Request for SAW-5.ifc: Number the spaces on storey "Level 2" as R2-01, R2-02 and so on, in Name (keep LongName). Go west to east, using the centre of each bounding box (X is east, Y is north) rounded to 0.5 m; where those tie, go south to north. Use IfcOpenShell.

First a look at what the model holds.

```python
import ifcopenshell
import ifcopenshell.util.element
import ifcopenshell.util.placement

model = ifcopenshell.open("SAW-5.ifc")
print(model.schema)
storey = next(s for s in model.by_type("IfcBuildingStorey") if s.Name == "Level 2")
spaces = [e for e in ifcopenshell.util.element.get_decomposition(storey) if e.is_a("IfcSpace")]
for e in sorted(spaces, key=lambda e: e.id()):
    origin = ifcopenshell.util.placement.get_local_placement(e.ObjectPlacement)[:3, 3]
    print(e.id(), e.Name, e.LongName, origin.round(2) + 0.0, sep=" | ")
```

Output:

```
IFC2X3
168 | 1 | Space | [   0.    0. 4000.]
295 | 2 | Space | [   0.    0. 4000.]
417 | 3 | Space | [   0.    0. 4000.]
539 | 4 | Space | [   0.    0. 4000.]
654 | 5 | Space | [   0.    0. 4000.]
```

```python
import ifcopenshell
import ifcopenshell.geom
import ifcopenshell.util.element
import ifcopenshell.util.shape

model = ifcopenshell.open("SAW-5.ifc")
settings = ifcopenshell.geom.settings()
settings.set("use-world-coords", True)


def centre(element):
    shape = ifcopenshell.geom.create_shape(settings, element)
    return ifcopenshell.util.shape.get_bbox_centroid(shape.geometry)


storey = next(s for s in model.by_type("IfcBuildingStorey") if s.Name == "Level 2")
spaces = [e for e in ifcopenshell.util.element.get_decomposition(storey) if e.is_a("IfcSpace")]

# Insertion points can sit at a corner or the storey origin, so sort by the geometry (in metres).
centres = {e: centre(e) for e in spaces}
spaces.sort(key=lambda e: (round(centres[e][0] / 0.5), centres[e][1]))

for i, e in enumerate(spaces, start=1):
    number = f"R2-{i:02d}"
    e.Name = number
    print(e.id(), number)

model.write("SAW-5_updated.ifc")
```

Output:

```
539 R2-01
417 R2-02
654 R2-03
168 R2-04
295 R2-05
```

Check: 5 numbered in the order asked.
